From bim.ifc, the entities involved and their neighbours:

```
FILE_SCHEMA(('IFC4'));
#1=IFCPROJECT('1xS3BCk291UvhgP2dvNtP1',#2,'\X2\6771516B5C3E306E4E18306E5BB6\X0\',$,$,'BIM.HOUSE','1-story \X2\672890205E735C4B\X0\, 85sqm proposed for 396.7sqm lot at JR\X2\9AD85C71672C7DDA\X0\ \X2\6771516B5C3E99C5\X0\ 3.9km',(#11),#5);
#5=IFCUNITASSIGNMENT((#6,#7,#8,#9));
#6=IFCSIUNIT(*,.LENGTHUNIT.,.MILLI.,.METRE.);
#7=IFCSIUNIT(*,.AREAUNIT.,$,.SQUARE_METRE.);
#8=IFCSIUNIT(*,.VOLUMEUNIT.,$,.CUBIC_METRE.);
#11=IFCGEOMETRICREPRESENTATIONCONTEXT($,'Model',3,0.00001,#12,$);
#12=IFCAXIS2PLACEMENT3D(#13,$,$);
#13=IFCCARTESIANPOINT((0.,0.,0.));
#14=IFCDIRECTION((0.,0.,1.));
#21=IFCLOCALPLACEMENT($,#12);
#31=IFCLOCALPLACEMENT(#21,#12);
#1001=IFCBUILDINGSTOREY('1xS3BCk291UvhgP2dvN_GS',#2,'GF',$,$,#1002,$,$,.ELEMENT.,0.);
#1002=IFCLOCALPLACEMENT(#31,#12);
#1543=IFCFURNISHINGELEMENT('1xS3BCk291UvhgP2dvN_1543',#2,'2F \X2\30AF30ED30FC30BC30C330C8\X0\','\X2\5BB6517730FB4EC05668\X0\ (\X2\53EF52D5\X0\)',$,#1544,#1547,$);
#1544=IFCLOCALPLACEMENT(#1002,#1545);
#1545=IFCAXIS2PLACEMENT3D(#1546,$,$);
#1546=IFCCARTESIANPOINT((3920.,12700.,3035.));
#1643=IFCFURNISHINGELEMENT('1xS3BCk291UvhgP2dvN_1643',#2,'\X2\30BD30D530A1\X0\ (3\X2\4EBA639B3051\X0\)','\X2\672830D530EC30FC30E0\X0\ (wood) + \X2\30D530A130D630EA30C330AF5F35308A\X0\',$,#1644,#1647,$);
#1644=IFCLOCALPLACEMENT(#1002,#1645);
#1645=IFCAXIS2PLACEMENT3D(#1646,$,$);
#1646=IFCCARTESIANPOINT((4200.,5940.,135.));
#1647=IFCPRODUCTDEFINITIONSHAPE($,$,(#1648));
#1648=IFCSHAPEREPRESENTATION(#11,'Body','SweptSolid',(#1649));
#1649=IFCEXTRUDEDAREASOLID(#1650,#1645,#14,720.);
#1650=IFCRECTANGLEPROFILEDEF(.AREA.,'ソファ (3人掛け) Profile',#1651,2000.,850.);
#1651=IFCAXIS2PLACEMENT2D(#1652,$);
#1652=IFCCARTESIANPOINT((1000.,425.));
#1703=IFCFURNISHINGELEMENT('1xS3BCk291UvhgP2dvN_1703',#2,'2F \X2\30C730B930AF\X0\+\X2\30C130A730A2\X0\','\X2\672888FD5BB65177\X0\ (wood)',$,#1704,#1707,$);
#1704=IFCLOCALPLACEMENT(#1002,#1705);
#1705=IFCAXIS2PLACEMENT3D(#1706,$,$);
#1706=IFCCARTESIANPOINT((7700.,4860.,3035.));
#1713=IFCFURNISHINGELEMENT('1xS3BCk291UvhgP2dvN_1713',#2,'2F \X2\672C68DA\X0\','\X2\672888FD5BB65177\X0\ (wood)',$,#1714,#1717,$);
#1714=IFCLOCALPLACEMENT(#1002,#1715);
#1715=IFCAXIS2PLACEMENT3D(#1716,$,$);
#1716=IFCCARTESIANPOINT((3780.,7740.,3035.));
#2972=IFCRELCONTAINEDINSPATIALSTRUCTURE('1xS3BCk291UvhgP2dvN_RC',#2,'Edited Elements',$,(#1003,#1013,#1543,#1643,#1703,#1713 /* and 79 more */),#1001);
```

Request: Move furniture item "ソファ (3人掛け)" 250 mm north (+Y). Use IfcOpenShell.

```python
import ifcopenshell
import ifcopenshell.api.geometry
import ifcopenshell.util.placement

model = ifcopenshell.open("bim.ifc")

item = model.by_guid("1xS3BCk291UvhgP2dvN_1643")
matrix = ifcopenshell.util.placement.get_local_placement(item.ObjectPlacement)
matrix[1, 3] += 250.0
ifcopenshell.api.geometry.edit_object_placement(model, product=item, matrix=matrix, is_si=False)

print(ifcopenshell.util.placement.get_local_placement(item.ObjectPlacement).round(3) + 0.0)

model.write("bim-out.ifc")
```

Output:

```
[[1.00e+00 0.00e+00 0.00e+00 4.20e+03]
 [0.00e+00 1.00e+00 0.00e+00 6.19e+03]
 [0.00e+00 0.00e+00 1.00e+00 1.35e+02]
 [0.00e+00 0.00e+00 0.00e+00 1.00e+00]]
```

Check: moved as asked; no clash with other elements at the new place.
